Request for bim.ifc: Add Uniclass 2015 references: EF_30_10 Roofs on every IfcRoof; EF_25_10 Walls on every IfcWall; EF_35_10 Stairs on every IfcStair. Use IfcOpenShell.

First a look at what the model holds.

```python
import ifcopenshell

model = ifcopenshell.open("bim.ifc")
print(model.schema)
print("classifications:", [c.Name for c in model.by_type("IfcClassification")])
for ifc_class in ("IfcDoor", "IfcRoof", "IfcStair", "IfcWall", "IfcWindow"):
    print(ifc_class, len(model.by_type(ifc_class)))
```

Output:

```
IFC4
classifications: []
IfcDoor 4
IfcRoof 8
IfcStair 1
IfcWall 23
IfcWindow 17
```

```python
import ifcopenshell
import ifcopenshell.api.classification

model = ifcopenshell.open("bim.ifc")

system = ifcopenshell.api.classification.add_classification(model, classification="Uniclass 2015")

codes = {
    "IfcRoof": ("EF_30_10", "Roofs"),
    "IfcWall": ("EF_25_10", "Walls"),
    "IfcStair": ("EF_35_10", "Stairs"),
}
for ifc_class, (code, name) in codes.items():
    products = model.by_type(ifc_class)
    ifcopenshell.api.classification.add_reference(
        model, products=products, classification=system, identification=code, name=name
    )
    print(code, len(products))

model.write("bim-out.ifc")
```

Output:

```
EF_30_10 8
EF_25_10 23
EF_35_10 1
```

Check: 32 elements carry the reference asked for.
